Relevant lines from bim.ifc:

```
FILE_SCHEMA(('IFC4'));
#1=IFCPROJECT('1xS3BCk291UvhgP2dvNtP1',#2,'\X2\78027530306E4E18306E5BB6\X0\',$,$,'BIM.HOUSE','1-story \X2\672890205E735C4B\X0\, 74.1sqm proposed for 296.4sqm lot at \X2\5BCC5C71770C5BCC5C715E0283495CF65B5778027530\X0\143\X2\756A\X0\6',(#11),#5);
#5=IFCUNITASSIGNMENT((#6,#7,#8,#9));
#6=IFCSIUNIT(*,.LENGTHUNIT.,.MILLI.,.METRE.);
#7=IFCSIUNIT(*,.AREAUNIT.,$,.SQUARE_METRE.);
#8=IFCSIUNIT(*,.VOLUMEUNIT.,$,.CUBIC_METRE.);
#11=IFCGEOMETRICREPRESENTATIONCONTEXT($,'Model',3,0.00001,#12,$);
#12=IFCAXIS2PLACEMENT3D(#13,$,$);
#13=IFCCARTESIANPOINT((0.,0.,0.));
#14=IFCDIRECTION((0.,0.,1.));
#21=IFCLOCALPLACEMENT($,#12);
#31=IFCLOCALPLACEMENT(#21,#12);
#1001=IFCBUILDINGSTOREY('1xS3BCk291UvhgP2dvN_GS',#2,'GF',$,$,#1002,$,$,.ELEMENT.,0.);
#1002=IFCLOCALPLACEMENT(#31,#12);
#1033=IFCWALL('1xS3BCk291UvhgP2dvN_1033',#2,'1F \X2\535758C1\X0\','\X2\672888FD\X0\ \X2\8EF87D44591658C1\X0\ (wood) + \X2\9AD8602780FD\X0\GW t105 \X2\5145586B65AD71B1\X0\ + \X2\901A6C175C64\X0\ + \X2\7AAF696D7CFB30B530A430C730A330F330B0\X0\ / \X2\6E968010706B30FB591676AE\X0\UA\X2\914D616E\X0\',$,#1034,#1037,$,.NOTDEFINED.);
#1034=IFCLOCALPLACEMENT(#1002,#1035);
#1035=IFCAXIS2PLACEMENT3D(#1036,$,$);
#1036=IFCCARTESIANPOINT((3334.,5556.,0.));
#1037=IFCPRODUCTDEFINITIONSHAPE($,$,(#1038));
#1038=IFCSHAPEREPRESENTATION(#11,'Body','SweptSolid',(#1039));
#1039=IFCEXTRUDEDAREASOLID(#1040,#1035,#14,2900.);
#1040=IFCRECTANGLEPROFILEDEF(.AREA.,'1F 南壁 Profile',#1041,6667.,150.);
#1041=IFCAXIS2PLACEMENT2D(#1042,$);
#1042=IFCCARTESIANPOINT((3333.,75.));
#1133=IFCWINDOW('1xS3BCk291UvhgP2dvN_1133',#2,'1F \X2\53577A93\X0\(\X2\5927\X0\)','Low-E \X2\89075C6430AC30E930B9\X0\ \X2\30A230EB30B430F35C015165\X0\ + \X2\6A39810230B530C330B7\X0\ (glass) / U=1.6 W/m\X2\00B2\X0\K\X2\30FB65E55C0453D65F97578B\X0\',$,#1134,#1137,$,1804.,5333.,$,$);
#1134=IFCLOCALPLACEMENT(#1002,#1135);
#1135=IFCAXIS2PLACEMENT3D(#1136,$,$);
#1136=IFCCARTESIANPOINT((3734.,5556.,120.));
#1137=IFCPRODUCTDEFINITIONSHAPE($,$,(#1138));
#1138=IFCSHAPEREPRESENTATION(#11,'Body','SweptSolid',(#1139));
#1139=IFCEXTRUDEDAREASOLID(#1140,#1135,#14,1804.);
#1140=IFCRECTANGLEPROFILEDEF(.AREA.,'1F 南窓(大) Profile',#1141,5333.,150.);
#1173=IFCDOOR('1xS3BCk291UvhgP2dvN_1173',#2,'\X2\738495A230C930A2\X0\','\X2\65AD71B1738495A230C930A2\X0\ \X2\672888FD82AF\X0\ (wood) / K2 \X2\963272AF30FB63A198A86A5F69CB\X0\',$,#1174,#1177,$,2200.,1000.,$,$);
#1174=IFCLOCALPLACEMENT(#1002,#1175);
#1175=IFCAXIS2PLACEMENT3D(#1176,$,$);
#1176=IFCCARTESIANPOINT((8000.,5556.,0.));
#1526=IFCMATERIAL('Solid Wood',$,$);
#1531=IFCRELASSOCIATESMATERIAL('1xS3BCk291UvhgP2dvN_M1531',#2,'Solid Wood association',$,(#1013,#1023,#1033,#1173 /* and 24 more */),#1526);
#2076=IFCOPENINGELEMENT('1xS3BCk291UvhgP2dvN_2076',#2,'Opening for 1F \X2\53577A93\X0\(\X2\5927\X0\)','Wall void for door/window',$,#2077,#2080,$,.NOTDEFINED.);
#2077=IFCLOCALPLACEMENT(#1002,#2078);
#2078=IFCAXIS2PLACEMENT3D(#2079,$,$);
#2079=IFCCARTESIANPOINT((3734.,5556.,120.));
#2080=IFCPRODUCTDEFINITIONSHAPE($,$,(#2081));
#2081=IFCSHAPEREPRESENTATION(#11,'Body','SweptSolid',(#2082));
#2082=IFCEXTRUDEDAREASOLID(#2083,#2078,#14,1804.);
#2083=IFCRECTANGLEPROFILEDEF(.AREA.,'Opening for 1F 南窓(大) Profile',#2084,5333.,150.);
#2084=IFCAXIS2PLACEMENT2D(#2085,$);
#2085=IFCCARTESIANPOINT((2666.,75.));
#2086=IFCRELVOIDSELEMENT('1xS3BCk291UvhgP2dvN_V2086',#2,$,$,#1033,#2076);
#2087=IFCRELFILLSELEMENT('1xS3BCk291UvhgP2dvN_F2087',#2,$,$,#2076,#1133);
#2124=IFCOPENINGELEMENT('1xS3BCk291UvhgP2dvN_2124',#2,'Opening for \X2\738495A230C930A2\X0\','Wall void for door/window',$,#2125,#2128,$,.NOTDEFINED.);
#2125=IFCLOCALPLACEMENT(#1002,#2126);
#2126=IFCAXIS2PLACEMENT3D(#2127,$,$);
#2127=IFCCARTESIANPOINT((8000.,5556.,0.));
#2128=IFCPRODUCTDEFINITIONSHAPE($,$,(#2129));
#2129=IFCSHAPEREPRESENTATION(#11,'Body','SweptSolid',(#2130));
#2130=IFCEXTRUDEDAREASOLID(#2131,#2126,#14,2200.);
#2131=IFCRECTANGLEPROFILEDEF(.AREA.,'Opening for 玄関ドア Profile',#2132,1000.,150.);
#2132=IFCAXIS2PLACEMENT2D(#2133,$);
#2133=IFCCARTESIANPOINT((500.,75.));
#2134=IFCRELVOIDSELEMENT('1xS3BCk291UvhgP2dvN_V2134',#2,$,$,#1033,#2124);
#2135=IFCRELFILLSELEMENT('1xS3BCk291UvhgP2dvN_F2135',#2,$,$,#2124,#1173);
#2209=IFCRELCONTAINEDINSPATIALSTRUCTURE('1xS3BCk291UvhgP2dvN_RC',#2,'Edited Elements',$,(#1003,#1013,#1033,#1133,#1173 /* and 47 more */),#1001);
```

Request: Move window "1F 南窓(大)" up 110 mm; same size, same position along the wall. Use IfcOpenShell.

```python
import numpy as np
import ifcopenshell
import ifcopenshell.api.geometry
import ifcopenshell.util.placement
import ifcopenshell.util.unit

model = ifcopenshell.open("bim.ifc")
unit_scale = ifcopenshell.util.unit.calculate_unit_scale(model)

window = model.by_guid("1xS3BCk291UvhgP2dvN_1133")
opening = window.FillsVoids[0].RelatingOpeningElement
dz = 0.11 / unit_scale

shift = np.array([0.0, 0.0, dz])
# The window is not placed relative to its opening, so move both.
for product in (opening, window):
    matrix = ifcopenshell.util.placement.get_local_placement(product.ObjectPlacement)
    matrix[:3, 3] += shift
    ifcopenshell.api.geometry.edit_object_placement(model, product=product, matrix=matrix, is_si=False)

print(f"moved by {dz * unit_scale:+.3f} m")

model.write("bim_v2.ifc")
```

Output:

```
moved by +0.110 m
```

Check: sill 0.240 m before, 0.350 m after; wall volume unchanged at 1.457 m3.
